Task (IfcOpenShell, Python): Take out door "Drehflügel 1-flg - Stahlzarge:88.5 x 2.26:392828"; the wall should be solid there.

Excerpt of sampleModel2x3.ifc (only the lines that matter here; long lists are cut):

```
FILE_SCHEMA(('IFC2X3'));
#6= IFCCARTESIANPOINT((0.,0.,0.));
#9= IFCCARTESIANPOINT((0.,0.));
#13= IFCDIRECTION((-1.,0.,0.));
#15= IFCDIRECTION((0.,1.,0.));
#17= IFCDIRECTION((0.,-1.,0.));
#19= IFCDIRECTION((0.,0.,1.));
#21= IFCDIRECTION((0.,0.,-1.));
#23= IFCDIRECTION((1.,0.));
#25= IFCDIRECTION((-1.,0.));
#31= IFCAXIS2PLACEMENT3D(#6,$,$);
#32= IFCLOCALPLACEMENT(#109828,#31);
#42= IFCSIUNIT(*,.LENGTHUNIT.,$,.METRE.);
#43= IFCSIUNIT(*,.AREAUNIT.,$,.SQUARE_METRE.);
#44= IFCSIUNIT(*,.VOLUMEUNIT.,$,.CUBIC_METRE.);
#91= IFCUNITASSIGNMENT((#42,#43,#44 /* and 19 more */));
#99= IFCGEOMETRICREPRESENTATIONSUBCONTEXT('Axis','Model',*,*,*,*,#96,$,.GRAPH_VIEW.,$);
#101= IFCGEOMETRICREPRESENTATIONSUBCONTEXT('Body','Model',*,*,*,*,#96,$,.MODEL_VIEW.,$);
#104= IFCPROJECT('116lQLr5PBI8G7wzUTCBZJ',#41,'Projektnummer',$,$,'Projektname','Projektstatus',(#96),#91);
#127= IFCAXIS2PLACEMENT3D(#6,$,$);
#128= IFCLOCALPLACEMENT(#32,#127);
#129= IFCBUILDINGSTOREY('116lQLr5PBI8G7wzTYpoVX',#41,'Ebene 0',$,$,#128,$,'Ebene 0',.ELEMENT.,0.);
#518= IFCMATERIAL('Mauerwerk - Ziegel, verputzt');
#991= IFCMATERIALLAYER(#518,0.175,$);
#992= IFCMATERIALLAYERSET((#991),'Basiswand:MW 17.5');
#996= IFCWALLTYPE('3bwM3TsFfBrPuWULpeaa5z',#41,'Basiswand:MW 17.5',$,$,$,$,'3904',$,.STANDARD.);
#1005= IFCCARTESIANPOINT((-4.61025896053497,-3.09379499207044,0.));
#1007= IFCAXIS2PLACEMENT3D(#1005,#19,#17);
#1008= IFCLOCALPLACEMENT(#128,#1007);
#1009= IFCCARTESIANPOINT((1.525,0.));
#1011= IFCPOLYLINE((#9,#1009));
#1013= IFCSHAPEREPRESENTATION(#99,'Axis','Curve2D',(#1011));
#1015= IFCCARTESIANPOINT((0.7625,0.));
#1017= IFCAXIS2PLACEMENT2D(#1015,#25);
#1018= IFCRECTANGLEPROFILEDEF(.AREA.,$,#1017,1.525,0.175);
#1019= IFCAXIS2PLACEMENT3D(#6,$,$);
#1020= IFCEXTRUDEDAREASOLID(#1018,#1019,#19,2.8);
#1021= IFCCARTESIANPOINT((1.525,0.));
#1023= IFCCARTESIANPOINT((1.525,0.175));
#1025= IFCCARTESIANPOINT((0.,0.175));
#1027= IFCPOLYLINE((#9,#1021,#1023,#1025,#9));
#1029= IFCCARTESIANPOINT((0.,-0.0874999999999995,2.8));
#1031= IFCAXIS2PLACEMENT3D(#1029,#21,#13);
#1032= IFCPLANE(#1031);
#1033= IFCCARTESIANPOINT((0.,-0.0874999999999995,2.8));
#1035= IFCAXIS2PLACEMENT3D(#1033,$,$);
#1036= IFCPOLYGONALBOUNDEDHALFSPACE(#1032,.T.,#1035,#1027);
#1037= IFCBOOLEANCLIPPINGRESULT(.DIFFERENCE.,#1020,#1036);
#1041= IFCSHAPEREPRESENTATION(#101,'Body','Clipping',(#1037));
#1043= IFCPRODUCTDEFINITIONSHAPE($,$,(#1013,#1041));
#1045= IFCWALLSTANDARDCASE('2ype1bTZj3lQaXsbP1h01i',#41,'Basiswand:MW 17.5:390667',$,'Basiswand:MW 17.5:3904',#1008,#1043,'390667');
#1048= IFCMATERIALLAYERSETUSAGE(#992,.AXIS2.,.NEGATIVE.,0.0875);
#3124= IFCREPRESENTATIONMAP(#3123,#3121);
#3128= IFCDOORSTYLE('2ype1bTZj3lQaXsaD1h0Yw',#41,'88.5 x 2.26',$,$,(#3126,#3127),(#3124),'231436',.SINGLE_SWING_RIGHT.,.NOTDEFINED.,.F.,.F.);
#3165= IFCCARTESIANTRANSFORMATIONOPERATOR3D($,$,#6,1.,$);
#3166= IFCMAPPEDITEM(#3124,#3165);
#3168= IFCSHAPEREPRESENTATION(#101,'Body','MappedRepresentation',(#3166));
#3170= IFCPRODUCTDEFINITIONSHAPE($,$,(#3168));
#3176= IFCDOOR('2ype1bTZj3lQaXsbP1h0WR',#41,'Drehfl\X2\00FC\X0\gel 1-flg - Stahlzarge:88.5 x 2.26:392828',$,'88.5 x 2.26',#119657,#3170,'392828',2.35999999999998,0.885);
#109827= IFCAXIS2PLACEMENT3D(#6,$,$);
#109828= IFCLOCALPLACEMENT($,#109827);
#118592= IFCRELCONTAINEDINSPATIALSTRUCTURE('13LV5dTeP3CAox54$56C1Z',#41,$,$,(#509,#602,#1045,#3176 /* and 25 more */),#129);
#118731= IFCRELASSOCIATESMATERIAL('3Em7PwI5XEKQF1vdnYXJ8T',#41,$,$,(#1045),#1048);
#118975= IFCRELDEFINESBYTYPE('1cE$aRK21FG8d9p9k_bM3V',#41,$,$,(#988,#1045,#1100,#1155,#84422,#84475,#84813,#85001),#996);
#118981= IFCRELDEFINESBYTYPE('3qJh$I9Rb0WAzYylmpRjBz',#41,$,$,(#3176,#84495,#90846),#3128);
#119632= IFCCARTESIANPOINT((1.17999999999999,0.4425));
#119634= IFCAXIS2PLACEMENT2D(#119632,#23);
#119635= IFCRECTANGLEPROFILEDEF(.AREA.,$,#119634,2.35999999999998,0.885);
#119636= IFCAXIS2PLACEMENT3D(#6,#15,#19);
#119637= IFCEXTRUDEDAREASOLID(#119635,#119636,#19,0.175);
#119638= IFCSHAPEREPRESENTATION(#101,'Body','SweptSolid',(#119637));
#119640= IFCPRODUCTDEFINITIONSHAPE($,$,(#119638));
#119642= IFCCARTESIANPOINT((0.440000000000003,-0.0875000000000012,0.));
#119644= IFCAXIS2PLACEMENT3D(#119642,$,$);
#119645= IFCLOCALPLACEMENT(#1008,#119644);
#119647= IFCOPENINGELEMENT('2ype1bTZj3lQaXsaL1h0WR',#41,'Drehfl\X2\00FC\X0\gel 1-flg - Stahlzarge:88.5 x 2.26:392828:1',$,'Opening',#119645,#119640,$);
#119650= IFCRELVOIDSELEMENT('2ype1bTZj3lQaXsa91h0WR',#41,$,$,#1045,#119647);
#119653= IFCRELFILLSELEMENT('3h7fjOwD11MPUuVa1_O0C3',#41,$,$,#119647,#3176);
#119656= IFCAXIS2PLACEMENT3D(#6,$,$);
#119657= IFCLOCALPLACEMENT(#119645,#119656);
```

```python
import ifcopenshell
import ifcopenshell.api.feature
import ifcopenshell.api.root
import ifcopenshell.geom
import ifcopenshell.util.shape

model = ifcopenshell.open("sampleModel2x3.ifc")
settings = ifcopenshell.geom.settings()


def volume(element):
    """Net volume in cubic metres, openings subtracted."""
    shape = ifcopenshell.geom.create_shape(settings, element)
    return ifcopenshell.util.shape.get_volume(shape.geometry)


door = model.by_guid("2ype1bTZj3lQaXsbP1h0WR")
opening = door.FillsVoids[0].RelatingOpeningElement
wall = opening.VoidsElements[0].RelatingBuildingElement
before = volume(wall)

ifcopenshell.api.root.remove_product(model, product=door)
ifcopenshell.api.feature.remove_feature(model, feature=opening)

after = volume(wall)

print(f"wall volume {before:.3f} -> {after:.3f} m3")

model.write("sampleModel2x3_rev.ifc")
```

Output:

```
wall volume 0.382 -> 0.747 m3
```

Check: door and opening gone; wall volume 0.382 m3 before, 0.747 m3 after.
